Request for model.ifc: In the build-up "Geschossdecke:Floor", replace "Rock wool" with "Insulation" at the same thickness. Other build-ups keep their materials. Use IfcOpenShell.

First a look at what the model holds.

```python
import ifcopenshell
import ifcopenshell.util.element

model = ifcopenshell.open("model.ifc")
print(model.schema)
for layer_set in model.by_type("IfcMaterialLayerSet"):
    if layer_set.LayerSetName == "Geschossdecke:Floor":
        for layer in layer_set.MaterialLayers:
            print(layer.id(), layer.Material and layer.Material.Name, layer.LayerThickness, sep=" | ")
        print(len(ifcopenshell.util.element.get_elements_by_material(model, layer_set)), "elements and types use it")
print(sorted(m.Name for m in model.by_type("IfcMaterial") if m.Name)[:60])
```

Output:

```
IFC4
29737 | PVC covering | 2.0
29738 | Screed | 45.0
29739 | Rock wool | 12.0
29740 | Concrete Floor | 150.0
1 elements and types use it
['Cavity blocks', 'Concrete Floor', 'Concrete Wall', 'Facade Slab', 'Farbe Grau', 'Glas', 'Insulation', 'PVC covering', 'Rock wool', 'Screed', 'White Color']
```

```python
import ifcopenshell
import ifcopenshell.api.material

model = ifcopenshell.open("model.ifc")

layer_set = next(s for s in model.by_type("IfcMaterialLayerSet") if s.LayerSetName == "Geschossdecke:Floor")
layer = next(l for l in layer_set.MaterialLayers if l.Material and l.Material.Name == "Rock wool")
material = next(m for m in model.by_type("IfcMaterial") if m.Name == "Insulation")

# Point this one layer at the other material; renaming the old one would change it everywhere.
ifcopenshell.api.material.edit_layer(model, layer=layer, attributes={}, material=material)

print([l.Material.Name if l.Material else None for l in layer_set.MaterialLayers])

model.write("model_edited.ifc")
```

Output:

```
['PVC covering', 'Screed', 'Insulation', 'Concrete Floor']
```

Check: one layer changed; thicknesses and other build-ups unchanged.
